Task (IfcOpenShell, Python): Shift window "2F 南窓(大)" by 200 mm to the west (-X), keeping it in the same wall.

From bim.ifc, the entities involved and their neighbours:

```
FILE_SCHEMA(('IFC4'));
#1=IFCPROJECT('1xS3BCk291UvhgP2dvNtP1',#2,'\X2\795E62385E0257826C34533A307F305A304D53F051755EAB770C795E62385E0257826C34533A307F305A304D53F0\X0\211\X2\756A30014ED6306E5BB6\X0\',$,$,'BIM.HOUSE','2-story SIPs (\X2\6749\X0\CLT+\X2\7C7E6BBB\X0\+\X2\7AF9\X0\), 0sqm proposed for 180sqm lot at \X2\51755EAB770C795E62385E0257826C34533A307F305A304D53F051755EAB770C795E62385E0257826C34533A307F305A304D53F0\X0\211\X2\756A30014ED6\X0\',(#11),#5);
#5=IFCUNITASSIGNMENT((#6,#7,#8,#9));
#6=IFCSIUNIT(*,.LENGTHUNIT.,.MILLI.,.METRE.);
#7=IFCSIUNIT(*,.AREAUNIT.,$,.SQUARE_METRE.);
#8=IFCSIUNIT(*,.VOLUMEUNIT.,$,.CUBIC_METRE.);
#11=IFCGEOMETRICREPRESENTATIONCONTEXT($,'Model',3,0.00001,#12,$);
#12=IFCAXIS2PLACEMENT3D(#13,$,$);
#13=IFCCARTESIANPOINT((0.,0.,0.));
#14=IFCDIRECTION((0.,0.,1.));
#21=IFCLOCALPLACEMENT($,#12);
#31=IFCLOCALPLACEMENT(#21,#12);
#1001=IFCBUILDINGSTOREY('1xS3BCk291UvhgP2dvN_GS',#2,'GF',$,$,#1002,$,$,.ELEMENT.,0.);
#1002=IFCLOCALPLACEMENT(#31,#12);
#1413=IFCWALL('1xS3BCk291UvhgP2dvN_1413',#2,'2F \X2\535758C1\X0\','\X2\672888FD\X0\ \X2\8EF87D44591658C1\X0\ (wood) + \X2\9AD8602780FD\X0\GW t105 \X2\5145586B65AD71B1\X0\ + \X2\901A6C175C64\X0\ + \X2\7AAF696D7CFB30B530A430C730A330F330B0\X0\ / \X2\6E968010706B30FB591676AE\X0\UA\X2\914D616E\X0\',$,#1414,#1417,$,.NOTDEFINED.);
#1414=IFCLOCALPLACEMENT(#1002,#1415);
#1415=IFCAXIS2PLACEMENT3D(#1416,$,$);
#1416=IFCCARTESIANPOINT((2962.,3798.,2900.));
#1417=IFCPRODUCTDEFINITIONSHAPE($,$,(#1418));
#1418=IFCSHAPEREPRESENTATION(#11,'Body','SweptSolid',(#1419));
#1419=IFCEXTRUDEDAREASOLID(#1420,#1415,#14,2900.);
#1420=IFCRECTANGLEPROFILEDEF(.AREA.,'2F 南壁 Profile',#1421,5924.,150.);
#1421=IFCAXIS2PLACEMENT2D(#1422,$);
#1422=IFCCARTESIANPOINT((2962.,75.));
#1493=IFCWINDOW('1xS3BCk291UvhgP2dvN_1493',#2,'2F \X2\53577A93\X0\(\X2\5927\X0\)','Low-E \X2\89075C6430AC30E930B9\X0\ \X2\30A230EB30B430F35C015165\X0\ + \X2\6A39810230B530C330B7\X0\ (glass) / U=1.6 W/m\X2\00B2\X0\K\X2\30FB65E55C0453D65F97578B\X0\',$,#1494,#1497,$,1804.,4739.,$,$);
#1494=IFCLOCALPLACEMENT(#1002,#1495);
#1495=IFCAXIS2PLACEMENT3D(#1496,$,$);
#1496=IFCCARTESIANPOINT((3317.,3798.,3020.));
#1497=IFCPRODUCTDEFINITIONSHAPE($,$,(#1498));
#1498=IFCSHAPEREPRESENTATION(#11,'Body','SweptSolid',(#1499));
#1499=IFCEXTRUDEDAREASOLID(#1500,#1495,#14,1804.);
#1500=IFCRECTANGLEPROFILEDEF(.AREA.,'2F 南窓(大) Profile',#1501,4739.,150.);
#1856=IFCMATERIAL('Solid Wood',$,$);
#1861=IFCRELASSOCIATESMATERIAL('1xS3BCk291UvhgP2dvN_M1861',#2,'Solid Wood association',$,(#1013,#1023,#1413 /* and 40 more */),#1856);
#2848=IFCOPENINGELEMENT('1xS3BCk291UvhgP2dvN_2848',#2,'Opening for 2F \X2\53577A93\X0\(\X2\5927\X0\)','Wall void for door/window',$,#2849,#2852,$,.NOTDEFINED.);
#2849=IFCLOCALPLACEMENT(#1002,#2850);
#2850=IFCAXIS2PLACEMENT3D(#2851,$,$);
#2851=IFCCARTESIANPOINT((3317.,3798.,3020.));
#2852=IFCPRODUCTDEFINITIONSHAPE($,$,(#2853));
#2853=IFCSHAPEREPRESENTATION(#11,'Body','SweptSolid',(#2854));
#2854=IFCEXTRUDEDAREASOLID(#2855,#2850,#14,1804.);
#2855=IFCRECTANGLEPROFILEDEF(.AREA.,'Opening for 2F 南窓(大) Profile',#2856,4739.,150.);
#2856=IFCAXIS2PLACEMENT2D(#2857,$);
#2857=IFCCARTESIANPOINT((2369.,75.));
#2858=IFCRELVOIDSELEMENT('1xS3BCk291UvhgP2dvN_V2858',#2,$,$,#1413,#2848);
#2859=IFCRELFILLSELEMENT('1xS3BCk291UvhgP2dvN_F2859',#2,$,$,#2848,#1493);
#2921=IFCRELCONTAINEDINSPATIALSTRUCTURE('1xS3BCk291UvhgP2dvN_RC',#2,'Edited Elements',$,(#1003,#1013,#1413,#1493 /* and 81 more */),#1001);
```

```python
import ifcopenshell
import ifcopenshell.api.geometry
import ifcopenshell.util.placement

model = ifcopenshell.open("bim.ifc")

window = model.by_id(1493)
opening = window.FillsVoids[0].RelatingOpeningElement
wall = opening.VoidsElements[0].RelatingBuildingElement

wall_matrix = ifcopenshell.util.placement.get_local_placement(wall.ObjectPlacement)
shift = wall_matrix[:3, 0] * -200.0
before = ifcopenshell.util.placement.get_local_placement(window.ObjectPlacement)[:3, 3].copy()

# The window is not placed relative to its opening, so move both.
for product in (opening, window):
    matrix = ifcopenshell.util.placement.get_local_placement(product.ObjectPlacement)
    matrix[:3, 3] += shift
    ifcopenshell.api.geometry.edit_object_placement(model, product=product, matrix=matrix, is_si=False)

after = ifcopenshell.util.placement.get_local_placement(window.ObjectPlacement)[:3, 3]
print("window moved by", (after - before).round(3) + 0.0)

model.write("bim-out.ifc")
```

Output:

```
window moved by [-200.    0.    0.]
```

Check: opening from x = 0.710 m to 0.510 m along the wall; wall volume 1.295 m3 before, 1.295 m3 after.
